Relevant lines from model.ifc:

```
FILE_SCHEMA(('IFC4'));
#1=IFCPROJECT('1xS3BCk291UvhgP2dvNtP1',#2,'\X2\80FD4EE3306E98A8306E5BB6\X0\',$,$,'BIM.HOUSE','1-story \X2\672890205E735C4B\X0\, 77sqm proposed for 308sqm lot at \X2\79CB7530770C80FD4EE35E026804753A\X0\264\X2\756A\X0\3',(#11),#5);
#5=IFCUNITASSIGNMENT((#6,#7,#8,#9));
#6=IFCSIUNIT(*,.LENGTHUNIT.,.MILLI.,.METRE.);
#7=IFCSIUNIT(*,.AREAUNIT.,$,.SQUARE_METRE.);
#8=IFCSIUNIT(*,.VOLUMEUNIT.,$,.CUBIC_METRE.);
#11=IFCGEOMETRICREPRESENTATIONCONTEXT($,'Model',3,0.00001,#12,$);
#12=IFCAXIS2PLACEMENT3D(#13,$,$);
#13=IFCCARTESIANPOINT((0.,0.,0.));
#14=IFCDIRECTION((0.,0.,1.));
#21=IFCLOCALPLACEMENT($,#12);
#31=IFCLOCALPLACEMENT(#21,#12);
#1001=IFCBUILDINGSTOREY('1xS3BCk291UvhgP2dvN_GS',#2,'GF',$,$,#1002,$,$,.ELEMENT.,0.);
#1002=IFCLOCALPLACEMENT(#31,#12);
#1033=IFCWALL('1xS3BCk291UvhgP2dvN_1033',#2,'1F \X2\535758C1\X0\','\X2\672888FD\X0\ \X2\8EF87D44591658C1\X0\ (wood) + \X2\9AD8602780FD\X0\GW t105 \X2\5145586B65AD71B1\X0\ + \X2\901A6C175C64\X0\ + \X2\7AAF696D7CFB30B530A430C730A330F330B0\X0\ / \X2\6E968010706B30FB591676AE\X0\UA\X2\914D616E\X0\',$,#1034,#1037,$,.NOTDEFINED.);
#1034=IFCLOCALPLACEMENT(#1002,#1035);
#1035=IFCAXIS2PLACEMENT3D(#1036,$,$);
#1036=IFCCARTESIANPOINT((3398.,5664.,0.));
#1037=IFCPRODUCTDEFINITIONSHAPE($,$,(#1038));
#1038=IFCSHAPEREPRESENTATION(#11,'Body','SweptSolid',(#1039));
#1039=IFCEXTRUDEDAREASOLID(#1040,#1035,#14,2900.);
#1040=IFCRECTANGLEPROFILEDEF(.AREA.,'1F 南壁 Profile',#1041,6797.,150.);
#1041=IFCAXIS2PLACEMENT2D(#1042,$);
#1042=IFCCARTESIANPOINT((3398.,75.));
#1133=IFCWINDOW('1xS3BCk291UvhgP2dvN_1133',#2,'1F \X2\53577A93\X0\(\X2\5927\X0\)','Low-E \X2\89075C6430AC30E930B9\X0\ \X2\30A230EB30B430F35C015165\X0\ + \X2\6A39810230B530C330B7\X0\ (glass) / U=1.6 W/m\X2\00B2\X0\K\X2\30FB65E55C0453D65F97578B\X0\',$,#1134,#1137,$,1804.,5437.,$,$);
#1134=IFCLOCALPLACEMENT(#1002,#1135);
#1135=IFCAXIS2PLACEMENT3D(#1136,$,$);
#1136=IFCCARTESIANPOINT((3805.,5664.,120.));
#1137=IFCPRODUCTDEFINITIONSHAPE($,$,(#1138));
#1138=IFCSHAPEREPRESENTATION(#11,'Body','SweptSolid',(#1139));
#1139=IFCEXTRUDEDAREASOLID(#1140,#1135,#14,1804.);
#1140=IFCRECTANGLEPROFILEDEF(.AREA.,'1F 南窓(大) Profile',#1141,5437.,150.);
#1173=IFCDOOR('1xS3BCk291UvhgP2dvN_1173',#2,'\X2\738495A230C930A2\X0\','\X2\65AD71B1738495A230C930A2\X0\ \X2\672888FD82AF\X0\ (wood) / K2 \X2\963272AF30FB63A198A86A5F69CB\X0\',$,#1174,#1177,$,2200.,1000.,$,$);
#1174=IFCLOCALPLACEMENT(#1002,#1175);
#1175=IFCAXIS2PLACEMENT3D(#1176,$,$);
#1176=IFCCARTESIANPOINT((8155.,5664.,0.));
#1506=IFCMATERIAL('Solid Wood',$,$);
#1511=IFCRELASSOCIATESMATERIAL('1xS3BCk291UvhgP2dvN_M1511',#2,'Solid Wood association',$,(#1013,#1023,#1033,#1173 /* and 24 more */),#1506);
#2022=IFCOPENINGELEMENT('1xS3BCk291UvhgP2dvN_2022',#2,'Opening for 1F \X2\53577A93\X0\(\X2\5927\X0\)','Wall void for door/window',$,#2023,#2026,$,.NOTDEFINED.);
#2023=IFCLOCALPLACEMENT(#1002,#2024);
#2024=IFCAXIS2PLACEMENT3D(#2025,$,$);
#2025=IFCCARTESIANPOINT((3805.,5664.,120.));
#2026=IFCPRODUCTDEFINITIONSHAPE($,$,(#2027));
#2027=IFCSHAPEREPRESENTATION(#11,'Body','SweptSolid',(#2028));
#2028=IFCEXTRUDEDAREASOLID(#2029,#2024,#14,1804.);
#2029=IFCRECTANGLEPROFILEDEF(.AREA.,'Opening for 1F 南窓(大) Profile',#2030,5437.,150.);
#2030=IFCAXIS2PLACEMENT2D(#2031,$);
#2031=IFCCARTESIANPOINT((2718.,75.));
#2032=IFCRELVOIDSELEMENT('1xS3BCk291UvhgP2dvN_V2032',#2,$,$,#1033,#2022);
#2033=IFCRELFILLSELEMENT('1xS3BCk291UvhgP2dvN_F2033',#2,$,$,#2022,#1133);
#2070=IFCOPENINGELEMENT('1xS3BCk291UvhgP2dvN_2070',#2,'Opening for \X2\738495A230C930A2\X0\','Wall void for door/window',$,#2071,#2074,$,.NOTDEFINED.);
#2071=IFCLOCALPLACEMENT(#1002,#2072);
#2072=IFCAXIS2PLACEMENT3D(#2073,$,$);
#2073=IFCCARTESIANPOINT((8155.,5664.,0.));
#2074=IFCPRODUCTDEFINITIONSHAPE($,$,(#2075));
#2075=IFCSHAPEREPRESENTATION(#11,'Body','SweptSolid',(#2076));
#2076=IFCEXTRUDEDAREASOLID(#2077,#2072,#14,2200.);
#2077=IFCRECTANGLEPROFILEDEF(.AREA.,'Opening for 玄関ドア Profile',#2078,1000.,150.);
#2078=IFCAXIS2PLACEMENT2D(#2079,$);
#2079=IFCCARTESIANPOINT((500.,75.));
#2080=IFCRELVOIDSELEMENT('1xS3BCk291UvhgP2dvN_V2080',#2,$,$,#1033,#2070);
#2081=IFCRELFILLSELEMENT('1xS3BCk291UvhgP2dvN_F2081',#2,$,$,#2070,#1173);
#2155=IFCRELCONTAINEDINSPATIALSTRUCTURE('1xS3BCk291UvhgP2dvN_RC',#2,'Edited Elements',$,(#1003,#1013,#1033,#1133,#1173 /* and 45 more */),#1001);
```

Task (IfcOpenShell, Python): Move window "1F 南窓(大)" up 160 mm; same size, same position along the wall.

```python
import numpy as np
import ifcopenshell
import ifcopenshell.api.geometry
import ifcopenshell.util.placement
import ifcopenshell.util.unit

model = ifcopenshell.open("model.ifc")
unit_scale = ifcopenshell.util.unit.calculate_unit_scale(model)

window = model.by_id(1133)
opening = window.FillsVoids[0].RelatingOpeningElement
dz = 0.16 / unit_scale

shift = np.array([0.0, 0.0, dz])
# The window is not placed relative to its opening, so move both.
for product in (opening, window):
    matrix = ifcopenshell.util.placement.get_local_placement(product.ObjectPlacement)
    matrix[:3, 3] += shift
    ifcopenshell.api.geometry.edit_object_placement(model, product=product, matrix=matrix, is_si=False)

print(f"moved by {dz * unit_scale:+.3f} m")

model.write("model_rev.ifc")
```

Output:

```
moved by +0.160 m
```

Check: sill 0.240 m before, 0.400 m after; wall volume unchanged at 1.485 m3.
